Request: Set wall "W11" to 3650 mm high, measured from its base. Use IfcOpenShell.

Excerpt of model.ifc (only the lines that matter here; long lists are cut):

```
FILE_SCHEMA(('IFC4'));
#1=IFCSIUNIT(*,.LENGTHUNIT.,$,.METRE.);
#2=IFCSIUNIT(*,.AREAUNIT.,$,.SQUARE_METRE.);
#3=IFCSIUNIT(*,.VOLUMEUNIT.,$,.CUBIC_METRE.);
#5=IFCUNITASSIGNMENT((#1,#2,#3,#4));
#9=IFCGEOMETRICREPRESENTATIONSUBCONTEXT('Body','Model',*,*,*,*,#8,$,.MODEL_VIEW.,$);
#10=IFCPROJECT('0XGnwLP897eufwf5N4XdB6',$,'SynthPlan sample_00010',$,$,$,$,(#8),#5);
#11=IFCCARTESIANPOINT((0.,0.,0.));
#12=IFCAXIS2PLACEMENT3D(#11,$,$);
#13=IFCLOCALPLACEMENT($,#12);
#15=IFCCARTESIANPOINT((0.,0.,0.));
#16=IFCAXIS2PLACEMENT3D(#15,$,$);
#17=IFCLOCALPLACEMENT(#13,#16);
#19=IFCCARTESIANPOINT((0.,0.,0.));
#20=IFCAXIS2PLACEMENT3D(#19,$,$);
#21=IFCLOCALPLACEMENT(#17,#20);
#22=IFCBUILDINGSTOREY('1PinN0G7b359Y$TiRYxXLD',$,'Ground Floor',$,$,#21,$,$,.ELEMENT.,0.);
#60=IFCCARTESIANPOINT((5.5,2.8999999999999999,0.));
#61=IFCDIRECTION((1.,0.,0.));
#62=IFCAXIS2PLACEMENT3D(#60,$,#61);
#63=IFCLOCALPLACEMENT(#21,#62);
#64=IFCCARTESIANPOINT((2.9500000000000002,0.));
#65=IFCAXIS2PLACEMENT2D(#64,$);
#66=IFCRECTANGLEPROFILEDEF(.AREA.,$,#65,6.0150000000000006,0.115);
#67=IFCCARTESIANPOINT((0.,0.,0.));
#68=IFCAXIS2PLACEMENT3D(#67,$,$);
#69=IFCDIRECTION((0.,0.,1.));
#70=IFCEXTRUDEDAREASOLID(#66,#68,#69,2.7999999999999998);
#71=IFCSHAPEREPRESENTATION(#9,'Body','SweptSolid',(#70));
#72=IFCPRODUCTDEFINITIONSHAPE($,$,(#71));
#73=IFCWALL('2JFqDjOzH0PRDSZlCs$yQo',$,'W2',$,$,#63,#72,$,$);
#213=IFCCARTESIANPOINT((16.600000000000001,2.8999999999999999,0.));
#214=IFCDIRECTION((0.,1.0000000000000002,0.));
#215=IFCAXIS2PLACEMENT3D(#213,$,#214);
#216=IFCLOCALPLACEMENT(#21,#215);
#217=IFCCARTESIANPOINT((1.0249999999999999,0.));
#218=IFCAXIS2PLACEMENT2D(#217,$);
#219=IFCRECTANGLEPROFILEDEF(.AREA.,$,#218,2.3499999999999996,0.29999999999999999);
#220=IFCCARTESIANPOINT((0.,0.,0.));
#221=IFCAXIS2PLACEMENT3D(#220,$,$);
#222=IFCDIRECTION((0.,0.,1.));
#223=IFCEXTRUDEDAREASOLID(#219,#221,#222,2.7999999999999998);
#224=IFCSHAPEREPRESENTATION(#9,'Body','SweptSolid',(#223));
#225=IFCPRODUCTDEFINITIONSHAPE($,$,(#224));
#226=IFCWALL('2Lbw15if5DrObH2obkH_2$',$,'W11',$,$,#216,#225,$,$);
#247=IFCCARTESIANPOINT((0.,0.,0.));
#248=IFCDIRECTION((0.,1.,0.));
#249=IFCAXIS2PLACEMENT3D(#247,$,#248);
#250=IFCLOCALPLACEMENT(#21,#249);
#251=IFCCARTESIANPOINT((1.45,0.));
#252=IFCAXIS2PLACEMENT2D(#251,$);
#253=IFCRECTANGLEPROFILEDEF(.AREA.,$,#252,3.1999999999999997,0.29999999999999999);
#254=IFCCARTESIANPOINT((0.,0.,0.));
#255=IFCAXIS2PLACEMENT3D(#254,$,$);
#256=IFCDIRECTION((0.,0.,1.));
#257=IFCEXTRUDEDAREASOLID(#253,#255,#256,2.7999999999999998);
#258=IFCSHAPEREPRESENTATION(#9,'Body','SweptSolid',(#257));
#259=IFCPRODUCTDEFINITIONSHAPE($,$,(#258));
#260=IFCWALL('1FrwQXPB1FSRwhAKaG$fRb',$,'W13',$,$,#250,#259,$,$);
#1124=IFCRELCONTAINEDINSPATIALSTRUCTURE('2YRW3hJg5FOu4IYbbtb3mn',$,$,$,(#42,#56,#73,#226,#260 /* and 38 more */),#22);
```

```python
import ifcopenshell
import ifcopenshell.geom
import ifcopenshell.util.representation
import ifcopenshell.util.shape
import ifcopenshell.util.unit

model = ifcopenshell.open("model.ifc")
unit_scale = ifcopenshell.util.unit.calculate_unit_scale(model)
settings = ifcopenshell.geom.settings()


def volume(element):
    """Net volume in cubic metres, openings subtracted."""
    shape = ifcopenshell.geom.create_shape(settings, element)
    return ifcopenshell.util.shape.get_volume(shape.geometry)


wall = model.by_guid("2Lbw15if5DrObH2obkH_2$")
before = volume(wall)

body = ifcopenshell.util.representation.get_representation(wall, "Model", "Body")
solid = body.Items[0]
old_height = solid.Depth
solid.Depth = 3.65 / unit_scale
after = volume(wall)

print(f"height {old_height:g} -> {solid.Depth:g}, volume {before:.3f} -> {after:.3f} m3")

model.write("model_v2.ifc")
```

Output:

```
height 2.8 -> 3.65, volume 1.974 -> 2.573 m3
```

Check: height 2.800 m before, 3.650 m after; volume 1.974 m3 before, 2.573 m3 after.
